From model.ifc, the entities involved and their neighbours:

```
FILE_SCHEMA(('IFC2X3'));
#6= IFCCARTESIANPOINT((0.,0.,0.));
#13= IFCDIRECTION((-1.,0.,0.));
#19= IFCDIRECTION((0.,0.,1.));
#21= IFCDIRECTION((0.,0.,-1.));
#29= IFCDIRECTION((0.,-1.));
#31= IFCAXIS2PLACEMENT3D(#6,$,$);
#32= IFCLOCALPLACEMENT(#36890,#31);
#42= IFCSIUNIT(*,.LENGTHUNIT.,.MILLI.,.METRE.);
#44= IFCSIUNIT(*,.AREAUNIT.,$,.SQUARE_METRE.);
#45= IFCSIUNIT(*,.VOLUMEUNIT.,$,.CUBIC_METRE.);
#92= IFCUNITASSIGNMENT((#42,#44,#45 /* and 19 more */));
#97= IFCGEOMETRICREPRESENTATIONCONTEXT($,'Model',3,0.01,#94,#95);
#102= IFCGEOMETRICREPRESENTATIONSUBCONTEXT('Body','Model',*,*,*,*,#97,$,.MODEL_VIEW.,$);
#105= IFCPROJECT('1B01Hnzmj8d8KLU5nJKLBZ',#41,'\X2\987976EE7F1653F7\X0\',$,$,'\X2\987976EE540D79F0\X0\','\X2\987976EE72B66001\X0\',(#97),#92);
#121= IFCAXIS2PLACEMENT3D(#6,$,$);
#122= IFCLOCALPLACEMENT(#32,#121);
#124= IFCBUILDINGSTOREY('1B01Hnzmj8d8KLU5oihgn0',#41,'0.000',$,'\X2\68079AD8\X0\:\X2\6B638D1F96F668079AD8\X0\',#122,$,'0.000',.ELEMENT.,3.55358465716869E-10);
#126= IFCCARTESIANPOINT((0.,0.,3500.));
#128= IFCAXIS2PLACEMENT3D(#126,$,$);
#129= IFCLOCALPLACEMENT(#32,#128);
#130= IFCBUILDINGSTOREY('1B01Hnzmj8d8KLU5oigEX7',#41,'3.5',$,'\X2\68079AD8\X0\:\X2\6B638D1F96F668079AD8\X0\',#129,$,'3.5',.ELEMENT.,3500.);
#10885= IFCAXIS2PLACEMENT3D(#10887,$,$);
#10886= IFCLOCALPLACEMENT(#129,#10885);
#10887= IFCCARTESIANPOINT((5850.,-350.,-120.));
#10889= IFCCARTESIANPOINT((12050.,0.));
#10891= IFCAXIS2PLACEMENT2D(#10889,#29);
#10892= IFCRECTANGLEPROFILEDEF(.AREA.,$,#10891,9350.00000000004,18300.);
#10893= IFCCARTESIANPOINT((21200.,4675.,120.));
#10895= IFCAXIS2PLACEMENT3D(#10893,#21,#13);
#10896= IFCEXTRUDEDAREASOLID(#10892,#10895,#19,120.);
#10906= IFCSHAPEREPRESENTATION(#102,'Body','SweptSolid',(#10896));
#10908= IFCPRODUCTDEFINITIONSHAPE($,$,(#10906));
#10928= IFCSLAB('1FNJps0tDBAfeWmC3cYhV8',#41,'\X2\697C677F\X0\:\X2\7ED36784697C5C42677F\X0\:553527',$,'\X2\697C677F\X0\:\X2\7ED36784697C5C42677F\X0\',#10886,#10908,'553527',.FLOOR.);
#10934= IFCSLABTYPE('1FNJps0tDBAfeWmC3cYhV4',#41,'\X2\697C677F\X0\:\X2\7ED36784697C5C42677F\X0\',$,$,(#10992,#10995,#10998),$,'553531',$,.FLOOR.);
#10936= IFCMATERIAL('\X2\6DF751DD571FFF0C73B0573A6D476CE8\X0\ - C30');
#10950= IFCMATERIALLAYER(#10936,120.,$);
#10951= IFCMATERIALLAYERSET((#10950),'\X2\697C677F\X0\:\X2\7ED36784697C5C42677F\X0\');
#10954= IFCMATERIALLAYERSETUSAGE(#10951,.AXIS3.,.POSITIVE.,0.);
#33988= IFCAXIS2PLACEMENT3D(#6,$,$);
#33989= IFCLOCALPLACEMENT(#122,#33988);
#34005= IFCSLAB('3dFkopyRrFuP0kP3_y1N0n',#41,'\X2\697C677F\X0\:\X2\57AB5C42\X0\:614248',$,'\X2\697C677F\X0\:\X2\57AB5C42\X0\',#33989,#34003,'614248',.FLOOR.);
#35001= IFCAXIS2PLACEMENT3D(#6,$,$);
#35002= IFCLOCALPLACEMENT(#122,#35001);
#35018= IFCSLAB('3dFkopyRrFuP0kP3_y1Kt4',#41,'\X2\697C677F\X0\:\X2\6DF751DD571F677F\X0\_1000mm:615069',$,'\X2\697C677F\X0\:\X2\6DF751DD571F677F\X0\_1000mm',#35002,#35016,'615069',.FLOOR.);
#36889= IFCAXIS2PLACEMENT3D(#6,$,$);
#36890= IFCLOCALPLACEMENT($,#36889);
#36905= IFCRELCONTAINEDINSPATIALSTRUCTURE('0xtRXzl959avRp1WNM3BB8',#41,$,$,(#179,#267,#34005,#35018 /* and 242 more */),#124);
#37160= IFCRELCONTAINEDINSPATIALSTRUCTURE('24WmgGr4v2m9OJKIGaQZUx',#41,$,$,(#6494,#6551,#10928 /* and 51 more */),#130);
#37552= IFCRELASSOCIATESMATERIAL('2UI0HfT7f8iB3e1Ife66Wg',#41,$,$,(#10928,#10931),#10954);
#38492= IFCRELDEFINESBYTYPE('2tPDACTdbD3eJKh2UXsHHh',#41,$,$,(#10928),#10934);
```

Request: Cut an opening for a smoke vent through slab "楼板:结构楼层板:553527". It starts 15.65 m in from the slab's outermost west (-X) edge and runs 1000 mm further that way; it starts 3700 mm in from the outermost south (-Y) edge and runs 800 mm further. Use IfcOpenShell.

```python
import numpy as np
import ifcopenshell
import ifcopenshell.api.feature
import ifcopenshell.api.geometry
import ifcopenshell.api.root
import ifcopenshell.geom
import ifcopenshell.util.placement
import ifcopenshell.util.representation
import ifcopenshell.util.shape
import ifcopenshell.util.unit

model = ifcopenshell.open("model.ifc")
unit_scale = ifcopenshell.util.unit.calculate_unit_scale(model)
settings = ifcopenshell.geom.settings()


def volume(element):
    """Net volume in cubic metres, openings subtracted."""
    shape = ifcopenshell.geom.create_shape(settings, element)
    return ifcopenshell.util.shape.get_volume(shape.geometry)


slab = model.by_id(10928)
before = volume(slab)

# Extent in the slab's own axes, in metres. The edges named are its -X and -Y sides.
slab_shape = ifcopenshell.geom.create_shape(settings, slab)
vertices = ifcopenshell.util.shape.get_vertices(slab_shape.geometry)
x_min, y_min, bottom = vertices.min(axis=0)
top = vertices[:, 2].max()

opening = ifcopenshell.api.root.create_entity(model, ifc_class="IfcOpeningElement", name="Smoke vent opening")
context = ifcopenshell.util.representation.get_context(model, "Model", "Body", "MODEL_VIEW")
width, depth = 1, 0.8
outline = [(0.0, 0.0), (width, 0.0), (width, depth), (0.0, depth), (0.0, 0.0)]
# Overshoot both faces by 50 mm so the cut is clean.
shape = ifcopenshell.api.geometry.add_slab_representation(
    model, context=context, depth=top - bottom + 0.1, polyline=outline
)
ifcopenshell.api.geometry.assign_representation(model, product=opening, representation=shape)

matrix = ifcopenshell.util.placement.get_local_placement(slab.ObjectPlacement)
matrix[:, 3] = matrix @ np.append(np.array([x_min + 15.65, y_min + 3.7, bottom - 0.05]) / unit_scale, 1.0)
ifcopenshell.api.geometry.edit_object_placement(model, product=opening, matrix=matrix, is_si=False)
ifcopenshell.api.feature.add_feature(model, feature=opening, element=slab)

after = volume(slab)

print(f"slab volume {before:.3f} -> {after:.3f} m3")

model.write("model_edited.ifc")
```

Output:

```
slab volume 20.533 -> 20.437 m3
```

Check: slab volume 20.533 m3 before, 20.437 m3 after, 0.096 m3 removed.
